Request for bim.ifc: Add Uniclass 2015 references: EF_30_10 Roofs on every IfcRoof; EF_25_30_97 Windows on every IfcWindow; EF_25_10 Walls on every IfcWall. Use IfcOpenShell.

First a look at what the model holds.

```python
import ifcopenshell

model = ifcopenshell.open("bim.ifc")
print(model.schema)
print("classifications:", [c.Name for c in model.by_type("IfcClassification")])
for ifc_class in ("IfcDoor", "IfcRoof", "IfcStair", "IfcWall", "IfcWindow"):
    print(ifc_class, len(model.by_type(ifc_class)))
```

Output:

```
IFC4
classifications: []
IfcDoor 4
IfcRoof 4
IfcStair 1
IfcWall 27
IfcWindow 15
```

```python
import ifcopenshell
import ifcopenshell.api.classification

model = ifcopenshell.open("bim.ifc")

system = ifcopenshell.api.classification.add_classification(model, classification="Uniclass 2015")

codes = {
    "IfcRoof": ("EF_30_10", "Roofs"),
    "IfcWindow": ("EF_25_30_97", "Windows"),
    "IfcWall": ("EF_25_10", "Walls"),
}
for ifc_class, (code, name) in codes.items():
    products = model.by_type(ifc_class)
    ifcopenshell.api.classification.add_reference(
        model, products=products, classification=system, identification=code, name=name
    )
    print(code, len(products))

model.write("bim_v2.ifc")
```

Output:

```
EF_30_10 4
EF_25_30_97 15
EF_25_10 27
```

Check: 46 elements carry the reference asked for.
